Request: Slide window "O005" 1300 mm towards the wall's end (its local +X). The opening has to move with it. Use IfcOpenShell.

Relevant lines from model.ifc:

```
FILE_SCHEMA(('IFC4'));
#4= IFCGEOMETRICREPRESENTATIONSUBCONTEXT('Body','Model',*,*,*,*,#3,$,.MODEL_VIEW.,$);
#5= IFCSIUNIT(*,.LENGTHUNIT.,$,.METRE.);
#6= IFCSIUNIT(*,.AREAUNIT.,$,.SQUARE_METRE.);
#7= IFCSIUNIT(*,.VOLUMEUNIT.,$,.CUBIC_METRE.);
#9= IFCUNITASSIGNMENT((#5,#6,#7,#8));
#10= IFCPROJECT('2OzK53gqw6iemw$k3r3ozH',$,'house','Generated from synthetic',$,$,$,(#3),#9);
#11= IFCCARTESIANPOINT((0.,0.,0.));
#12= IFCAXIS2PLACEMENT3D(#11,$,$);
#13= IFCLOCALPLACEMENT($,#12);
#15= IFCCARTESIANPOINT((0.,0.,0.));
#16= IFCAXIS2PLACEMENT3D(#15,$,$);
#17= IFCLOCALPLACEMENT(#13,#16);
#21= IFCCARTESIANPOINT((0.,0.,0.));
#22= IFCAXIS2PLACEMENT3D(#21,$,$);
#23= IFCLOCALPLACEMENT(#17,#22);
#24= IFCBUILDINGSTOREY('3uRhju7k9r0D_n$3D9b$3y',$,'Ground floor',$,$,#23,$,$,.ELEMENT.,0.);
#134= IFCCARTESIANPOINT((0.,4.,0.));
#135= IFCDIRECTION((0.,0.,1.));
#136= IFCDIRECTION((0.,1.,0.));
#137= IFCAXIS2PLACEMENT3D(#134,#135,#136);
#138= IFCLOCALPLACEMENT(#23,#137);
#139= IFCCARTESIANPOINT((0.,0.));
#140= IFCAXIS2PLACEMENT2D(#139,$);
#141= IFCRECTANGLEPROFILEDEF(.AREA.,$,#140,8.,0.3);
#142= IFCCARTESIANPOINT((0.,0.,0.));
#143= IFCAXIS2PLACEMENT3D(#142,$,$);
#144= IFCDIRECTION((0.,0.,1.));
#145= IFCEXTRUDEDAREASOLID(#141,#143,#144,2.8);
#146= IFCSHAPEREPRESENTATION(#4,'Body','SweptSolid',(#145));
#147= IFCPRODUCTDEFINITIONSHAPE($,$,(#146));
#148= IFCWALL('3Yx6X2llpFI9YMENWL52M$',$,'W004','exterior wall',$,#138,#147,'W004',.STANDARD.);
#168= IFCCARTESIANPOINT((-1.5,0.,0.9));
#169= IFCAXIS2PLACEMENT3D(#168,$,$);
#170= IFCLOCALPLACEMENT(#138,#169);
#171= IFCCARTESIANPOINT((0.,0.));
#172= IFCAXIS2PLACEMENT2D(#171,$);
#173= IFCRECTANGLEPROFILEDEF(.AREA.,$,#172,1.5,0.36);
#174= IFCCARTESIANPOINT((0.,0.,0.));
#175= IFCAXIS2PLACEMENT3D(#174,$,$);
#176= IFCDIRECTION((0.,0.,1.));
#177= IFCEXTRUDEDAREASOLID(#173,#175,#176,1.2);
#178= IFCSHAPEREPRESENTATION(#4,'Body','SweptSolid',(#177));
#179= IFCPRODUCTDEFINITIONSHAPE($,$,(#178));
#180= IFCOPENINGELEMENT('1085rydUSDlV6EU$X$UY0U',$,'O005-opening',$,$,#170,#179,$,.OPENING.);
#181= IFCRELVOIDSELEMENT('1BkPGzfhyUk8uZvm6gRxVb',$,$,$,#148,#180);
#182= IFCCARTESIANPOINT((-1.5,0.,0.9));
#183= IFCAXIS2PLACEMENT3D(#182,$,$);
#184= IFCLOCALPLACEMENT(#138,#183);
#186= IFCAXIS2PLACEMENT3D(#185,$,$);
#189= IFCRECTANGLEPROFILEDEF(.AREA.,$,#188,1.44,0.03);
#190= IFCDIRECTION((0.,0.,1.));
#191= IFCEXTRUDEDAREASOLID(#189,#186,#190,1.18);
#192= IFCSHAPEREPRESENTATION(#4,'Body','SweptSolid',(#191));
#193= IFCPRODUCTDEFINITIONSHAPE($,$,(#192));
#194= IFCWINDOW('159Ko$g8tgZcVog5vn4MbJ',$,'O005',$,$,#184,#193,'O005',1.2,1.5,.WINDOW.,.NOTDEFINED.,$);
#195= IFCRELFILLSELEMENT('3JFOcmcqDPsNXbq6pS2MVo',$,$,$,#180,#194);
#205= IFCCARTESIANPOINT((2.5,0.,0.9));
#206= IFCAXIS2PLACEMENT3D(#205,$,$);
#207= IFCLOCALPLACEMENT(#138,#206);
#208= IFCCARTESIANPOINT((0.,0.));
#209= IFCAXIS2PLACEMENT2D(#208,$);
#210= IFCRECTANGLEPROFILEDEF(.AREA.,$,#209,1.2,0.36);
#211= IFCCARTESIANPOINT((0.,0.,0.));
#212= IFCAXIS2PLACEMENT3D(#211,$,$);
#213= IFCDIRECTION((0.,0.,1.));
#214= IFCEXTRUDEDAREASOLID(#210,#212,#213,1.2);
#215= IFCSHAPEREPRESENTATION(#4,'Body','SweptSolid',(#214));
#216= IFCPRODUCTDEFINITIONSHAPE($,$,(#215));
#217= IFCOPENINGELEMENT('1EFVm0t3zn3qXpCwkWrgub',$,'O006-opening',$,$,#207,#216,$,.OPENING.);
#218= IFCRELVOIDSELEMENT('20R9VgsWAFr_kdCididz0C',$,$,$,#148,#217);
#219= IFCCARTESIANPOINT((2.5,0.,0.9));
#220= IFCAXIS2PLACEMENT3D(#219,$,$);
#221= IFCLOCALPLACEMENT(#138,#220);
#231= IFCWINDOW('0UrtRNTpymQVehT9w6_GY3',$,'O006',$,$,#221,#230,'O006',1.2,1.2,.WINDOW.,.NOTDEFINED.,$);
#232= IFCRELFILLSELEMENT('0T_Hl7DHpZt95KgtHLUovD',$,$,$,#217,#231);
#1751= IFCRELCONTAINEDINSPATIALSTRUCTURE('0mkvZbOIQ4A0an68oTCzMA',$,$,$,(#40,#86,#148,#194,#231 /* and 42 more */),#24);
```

```python
import ifcopenshell
import ifcopenshell.api.geometry
import ifcopenshell.util.placement
import ifcopenshell.util.unit

model = ifcopenshell.open("model.ifc")
unit_scale = ifcopenshell.util.unit.calculate_unit_scale(model)

window = model.by_id(194)
opening = window.FillsVoids[0].RelatingOpeningElement
wall = opening.VoidsElements[0].RelatingBuildingElement

wall_matrix = ifcopenshell.util.placement.get_local_placement(wall.ObjectPlacement)
shift = wall_matrix[:3, 0] * 1.3 / unit_scale
before = ifcopenshell.util.placement.get_local_placement(window.ObjectPlacement)[:3, 3].copy()

# The window is not placed relative to its opening, so move both.
for product in (opening, window):
    matrix = ifcopenshell.util.placement.get_local_placement(product.ObjectPlacement)
    matrix[:3, 3] += shift
    ifcopenshell.api.geometry.edit_object_placement(model, product=product, matrix=matrix, is_si=False)

after = ifcopenshell.util.placement.get_local_placement(window.ObjectPlacement)[:3, 3]
print("window moved by", (after - before).round(3) + 0.0)

model.write("model_rev.ifc")
```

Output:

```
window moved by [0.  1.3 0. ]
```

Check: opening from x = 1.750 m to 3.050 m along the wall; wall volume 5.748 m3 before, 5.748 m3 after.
